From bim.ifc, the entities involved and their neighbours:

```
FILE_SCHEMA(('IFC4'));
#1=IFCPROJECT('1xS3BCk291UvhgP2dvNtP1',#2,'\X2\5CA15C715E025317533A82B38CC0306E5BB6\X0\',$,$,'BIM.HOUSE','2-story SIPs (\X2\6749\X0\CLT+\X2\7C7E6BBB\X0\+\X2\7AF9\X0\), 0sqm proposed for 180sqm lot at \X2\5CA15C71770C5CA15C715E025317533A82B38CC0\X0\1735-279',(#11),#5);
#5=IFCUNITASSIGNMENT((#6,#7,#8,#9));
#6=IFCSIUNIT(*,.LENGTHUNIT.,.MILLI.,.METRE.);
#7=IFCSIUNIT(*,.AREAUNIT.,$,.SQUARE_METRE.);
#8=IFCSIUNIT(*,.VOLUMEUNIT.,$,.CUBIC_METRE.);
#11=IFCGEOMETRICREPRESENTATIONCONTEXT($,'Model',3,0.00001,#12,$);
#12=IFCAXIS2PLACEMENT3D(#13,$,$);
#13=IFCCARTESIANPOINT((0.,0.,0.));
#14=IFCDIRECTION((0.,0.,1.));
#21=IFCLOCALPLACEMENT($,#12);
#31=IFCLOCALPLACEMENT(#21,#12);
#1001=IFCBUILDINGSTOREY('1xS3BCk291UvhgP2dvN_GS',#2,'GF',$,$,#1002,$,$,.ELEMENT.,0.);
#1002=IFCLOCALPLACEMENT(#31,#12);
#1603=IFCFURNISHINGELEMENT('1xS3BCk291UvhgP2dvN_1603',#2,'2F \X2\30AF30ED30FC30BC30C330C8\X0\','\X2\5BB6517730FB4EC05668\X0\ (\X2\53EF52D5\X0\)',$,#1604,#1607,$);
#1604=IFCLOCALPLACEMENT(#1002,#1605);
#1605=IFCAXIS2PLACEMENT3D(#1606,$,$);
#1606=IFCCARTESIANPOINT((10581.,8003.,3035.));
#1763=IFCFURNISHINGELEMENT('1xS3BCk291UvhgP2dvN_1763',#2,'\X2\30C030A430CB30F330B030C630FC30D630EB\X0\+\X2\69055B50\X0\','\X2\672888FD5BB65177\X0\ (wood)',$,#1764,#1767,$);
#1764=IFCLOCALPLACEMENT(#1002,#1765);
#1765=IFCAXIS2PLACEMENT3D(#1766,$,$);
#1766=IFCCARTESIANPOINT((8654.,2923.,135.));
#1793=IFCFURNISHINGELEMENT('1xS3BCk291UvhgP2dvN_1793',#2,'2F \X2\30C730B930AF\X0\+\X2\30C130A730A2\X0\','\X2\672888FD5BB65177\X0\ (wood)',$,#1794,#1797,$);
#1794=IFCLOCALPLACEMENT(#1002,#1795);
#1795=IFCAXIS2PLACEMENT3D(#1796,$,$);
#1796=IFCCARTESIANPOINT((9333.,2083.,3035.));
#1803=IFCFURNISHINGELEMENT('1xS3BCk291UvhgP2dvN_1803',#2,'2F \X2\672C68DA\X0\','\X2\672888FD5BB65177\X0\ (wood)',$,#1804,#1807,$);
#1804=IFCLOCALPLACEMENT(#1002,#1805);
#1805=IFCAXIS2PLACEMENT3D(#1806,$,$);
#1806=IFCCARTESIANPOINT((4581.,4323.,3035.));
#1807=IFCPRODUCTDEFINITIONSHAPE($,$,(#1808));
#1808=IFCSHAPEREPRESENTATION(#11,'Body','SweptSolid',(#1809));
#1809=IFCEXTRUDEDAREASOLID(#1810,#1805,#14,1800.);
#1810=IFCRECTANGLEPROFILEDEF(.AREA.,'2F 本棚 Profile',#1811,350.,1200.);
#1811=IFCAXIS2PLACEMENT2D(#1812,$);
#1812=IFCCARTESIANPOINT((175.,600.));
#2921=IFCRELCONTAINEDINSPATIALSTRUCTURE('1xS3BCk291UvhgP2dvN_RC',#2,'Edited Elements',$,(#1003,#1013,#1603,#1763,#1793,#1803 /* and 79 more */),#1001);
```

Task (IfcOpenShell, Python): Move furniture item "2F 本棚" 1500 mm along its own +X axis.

```python
import ifcopenshell
import ifcopenshell.api.geometry
import ifcopenshell.util.placement
import ifcopenshell.util.unit

model = ifcopenshell.open("bim.ifc")
unit_scale = ifcopenshell.util.unit.calculate_unit_scale(model)

item = model.by_id(1803)
matrix = ifcopenshell.util.placement.get_local_placement(item.ObjectPlacement)
matrix[:3, 3] += matrix[:3, 0] * 1.5 / unit_scale
ifcopenshell.api.geometry.edit_object_placement(model, product=item, matrix=matrix, is_si=False)

print(ifcopenshell.util.placement.get_local_placement(item.ObjectPlacement).round(3) + 0.0)

model.write("bim_updated.ifc")
```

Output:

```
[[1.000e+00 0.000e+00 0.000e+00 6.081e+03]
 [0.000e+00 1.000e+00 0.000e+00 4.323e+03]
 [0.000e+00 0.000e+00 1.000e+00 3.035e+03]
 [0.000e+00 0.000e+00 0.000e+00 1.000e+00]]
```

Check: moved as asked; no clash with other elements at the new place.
